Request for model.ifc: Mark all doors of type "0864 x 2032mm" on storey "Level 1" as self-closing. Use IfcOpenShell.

First a look at what the model holds.

```python
import ifcopenshell
import ifcopenshell.util.element

model = ifcopenshell.open("model.ifc")
print(model.schema)
storey = next(s for s in model.by_type("IfcBuildingStorey") if s.Name == "Level 1")
doors = [e for e in ifcopenshell.util.element.get_decomposition(storey) if e.is_a("IfcDoor")]
seen = {}
for e in doors:
    element_type = ifcopenshell.util.element.get_type(e)
    key = (element_type.Name if element_type != e and element_type else None, ifcopenshell.util.element.get_pset(e, "Pset_DoorCommon", "SelfClosing"))
    seen[key] = seen.get(key, 0) + 1
for (name, value), count in sorted(seen.items(), key=str):
    print(count, "x", name, "|", value)
```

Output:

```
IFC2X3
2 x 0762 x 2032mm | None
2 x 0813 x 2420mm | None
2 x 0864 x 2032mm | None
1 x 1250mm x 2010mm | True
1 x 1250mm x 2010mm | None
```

```python
import ifcopenshell
import ifcopenshell.api.pset
import ifcopenshell.util.element

model = ifcopenshell.open("model.ifc")

storey = next(s for s in model.by_type("IfcBuildingStorey") if s.Name == "Level 1")
doors = [e for e in ifcopenshell.util.element.get_decomposition(storey) if e.is_a("IfcDoor")]

count = 0
for e in doors:
    element_type = ifcopenshell.util.element.get_type(e)
    if element_type in (None, e) or element_type.Name != "0864 x 2032mm":
        continue
    # add_pset returns the element's existing set when there is one.
    pset = ifcopenshell.api.pset.add_pset(model, product=e, name="Pset_DoorCommon")
    ifcopenshell.api.pset.edit_pset(model, pset=pset, properties={"SelfClosing": True})
    count += 1

print(count, "doors updated")

model.write("model_v2.ifc")
```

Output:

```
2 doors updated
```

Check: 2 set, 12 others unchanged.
